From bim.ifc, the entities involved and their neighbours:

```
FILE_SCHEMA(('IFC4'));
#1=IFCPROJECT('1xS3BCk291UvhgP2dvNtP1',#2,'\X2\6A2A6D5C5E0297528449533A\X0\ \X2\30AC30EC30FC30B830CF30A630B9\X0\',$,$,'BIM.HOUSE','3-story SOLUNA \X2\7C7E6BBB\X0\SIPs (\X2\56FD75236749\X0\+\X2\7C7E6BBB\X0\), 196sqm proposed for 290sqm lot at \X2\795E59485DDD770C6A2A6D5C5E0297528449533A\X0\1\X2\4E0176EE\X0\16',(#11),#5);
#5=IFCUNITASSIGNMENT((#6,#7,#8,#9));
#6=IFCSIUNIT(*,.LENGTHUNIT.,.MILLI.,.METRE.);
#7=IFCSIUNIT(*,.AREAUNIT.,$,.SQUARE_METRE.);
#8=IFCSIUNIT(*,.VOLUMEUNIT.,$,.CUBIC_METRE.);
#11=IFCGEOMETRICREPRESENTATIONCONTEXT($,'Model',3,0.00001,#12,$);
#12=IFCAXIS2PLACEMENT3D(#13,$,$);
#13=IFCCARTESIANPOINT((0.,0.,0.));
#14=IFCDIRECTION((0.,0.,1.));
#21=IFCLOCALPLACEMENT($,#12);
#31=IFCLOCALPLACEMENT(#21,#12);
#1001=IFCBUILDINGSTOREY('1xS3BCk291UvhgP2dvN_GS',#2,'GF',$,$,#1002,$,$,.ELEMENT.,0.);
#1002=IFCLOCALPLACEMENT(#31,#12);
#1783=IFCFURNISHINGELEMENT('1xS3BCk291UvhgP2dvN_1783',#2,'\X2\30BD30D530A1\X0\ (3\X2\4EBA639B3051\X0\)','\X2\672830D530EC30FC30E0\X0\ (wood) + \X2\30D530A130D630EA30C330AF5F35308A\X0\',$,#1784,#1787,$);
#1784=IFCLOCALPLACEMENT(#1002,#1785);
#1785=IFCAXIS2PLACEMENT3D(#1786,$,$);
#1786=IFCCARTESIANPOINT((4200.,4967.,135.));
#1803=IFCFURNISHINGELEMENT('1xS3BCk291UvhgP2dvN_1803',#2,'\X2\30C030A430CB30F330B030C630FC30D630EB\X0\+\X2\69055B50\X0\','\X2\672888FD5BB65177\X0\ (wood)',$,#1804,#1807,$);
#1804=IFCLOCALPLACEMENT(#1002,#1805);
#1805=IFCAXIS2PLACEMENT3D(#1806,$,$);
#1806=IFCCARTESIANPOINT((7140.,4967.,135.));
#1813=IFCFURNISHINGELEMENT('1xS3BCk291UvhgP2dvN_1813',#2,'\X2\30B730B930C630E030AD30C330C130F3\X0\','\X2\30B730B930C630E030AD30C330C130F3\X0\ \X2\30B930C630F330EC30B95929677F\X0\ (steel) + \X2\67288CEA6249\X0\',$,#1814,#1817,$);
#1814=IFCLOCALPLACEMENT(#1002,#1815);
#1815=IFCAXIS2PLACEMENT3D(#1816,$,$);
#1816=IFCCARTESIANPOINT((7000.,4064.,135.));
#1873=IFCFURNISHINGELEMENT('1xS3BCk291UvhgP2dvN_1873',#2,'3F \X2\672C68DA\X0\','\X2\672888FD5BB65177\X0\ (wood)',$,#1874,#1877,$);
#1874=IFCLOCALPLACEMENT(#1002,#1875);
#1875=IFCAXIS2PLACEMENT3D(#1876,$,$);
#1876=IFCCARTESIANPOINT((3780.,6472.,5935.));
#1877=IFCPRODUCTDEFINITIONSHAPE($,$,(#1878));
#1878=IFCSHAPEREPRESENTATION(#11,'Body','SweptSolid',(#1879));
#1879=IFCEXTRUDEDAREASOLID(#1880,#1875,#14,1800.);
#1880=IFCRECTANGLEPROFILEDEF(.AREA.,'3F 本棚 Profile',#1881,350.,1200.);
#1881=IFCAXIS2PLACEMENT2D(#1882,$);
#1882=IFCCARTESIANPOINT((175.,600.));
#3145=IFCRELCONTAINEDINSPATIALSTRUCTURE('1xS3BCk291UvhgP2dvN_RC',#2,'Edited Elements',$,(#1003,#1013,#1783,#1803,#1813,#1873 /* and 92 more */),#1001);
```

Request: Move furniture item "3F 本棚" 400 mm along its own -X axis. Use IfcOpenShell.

```python
import ifcopenshell
import ifcopenshell.api.geometry
import ifcopenshell.util.placement

model = ifcopenshell.open("bim.ifc")

item = model.by_guid("1xS3BCk291UvhgP2dvN_1873")
matrix = ifcopenshell.util.placement.get_local_placement(item.ObjectPlacement)
matrix[:3, 3] -= matrix[:3, 0] * 400.0
ifcopenshell.api.geometry.edit_object_placement(model, product=item, matrix=matrix, is_si=False)

print(ifcopenshell.util.placement.get_local_placement(item.ObjectPlacement).round(3) + 0.0)

model.write("bim_v2.ifc")
```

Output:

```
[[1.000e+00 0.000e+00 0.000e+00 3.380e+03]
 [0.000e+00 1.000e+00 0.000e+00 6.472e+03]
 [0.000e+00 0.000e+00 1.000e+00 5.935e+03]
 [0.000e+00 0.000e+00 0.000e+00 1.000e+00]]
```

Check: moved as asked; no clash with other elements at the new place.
